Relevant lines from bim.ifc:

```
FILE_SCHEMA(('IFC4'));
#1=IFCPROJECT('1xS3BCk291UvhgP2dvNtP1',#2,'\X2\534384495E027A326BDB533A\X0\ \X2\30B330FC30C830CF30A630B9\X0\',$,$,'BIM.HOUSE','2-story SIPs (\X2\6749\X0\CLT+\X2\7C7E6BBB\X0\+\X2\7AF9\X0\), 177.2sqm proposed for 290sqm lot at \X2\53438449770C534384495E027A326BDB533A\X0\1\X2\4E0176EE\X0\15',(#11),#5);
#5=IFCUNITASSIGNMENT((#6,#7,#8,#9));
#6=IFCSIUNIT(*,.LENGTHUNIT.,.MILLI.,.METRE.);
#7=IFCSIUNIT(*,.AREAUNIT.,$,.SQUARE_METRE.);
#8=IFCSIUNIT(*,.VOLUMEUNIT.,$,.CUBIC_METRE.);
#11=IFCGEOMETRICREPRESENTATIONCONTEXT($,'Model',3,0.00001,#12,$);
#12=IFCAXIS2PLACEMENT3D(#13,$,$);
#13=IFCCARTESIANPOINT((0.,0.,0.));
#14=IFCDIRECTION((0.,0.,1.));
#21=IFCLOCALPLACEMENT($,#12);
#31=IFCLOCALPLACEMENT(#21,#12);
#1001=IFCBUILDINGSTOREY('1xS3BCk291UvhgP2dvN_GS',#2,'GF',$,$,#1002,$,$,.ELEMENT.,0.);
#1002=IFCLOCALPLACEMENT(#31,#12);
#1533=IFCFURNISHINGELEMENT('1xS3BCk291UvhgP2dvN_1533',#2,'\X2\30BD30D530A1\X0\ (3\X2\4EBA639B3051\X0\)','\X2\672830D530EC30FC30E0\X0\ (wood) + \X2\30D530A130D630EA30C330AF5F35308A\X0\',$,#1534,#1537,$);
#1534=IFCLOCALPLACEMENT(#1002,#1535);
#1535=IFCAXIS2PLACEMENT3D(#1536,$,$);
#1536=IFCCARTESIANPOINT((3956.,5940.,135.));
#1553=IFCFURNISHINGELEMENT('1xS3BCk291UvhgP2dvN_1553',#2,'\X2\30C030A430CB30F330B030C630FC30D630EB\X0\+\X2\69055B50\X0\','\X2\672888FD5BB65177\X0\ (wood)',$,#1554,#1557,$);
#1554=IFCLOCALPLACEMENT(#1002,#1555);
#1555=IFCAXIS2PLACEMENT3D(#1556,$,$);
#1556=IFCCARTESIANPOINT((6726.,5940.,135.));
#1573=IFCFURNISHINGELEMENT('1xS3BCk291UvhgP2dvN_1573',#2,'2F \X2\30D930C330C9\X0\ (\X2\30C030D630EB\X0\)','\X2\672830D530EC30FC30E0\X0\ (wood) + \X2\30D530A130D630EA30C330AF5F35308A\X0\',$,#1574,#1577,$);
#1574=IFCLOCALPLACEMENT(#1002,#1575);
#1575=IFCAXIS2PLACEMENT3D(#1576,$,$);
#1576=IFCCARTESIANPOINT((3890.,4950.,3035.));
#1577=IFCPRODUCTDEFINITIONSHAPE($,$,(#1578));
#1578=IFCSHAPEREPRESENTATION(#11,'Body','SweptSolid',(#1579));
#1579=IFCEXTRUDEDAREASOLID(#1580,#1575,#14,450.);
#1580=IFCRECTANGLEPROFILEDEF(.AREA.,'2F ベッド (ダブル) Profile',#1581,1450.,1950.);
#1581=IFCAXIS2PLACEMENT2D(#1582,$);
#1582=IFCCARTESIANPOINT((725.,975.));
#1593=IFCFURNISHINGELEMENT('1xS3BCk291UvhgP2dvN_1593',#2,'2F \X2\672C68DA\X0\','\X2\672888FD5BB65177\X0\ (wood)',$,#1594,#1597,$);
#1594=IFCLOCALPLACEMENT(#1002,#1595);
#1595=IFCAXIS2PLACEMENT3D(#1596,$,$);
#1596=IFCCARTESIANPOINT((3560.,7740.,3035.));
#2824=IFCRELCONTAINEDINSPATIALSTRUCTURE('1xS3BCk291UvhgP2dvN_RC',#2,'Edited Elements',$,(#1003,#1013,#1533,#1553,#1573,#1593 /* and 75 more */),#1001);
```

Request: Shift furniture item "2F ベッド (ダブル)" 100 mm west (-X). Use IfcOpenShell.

```python
import ifcopenshell
import ifcopenshell.api.geometry
import ifcopenshell.util.placement
import ifcopenshell.util.unit

model = ifcopenshell.open("bim.ifc")
unit_scale = ifcopenshell.util.unit.calculate_unit_scale(model)

item = model.by_id(1573)
matrix = ifcopenshell.util.placement.get_local_placement(item.ObjectPlacement)
matrix[0, 3] -= 0.1 / unit_scale
ifcopenshell.api.geometry.edit_object_placement(model, product=item, matrix=matrix, is_si=False)

print(ifcopenshell.util.placement.get_local_placement(item.ObjectPlacement).round(3) + 0.0)

model.write("bim_edited.ifc")
```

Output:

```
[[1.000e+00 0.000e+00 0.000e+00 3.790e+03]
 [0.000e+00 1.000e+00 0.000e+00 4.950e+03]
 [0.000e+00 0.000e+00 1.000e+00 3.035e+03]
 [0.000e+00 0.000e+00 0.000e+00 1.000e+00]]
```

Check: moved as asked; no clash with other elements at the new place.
